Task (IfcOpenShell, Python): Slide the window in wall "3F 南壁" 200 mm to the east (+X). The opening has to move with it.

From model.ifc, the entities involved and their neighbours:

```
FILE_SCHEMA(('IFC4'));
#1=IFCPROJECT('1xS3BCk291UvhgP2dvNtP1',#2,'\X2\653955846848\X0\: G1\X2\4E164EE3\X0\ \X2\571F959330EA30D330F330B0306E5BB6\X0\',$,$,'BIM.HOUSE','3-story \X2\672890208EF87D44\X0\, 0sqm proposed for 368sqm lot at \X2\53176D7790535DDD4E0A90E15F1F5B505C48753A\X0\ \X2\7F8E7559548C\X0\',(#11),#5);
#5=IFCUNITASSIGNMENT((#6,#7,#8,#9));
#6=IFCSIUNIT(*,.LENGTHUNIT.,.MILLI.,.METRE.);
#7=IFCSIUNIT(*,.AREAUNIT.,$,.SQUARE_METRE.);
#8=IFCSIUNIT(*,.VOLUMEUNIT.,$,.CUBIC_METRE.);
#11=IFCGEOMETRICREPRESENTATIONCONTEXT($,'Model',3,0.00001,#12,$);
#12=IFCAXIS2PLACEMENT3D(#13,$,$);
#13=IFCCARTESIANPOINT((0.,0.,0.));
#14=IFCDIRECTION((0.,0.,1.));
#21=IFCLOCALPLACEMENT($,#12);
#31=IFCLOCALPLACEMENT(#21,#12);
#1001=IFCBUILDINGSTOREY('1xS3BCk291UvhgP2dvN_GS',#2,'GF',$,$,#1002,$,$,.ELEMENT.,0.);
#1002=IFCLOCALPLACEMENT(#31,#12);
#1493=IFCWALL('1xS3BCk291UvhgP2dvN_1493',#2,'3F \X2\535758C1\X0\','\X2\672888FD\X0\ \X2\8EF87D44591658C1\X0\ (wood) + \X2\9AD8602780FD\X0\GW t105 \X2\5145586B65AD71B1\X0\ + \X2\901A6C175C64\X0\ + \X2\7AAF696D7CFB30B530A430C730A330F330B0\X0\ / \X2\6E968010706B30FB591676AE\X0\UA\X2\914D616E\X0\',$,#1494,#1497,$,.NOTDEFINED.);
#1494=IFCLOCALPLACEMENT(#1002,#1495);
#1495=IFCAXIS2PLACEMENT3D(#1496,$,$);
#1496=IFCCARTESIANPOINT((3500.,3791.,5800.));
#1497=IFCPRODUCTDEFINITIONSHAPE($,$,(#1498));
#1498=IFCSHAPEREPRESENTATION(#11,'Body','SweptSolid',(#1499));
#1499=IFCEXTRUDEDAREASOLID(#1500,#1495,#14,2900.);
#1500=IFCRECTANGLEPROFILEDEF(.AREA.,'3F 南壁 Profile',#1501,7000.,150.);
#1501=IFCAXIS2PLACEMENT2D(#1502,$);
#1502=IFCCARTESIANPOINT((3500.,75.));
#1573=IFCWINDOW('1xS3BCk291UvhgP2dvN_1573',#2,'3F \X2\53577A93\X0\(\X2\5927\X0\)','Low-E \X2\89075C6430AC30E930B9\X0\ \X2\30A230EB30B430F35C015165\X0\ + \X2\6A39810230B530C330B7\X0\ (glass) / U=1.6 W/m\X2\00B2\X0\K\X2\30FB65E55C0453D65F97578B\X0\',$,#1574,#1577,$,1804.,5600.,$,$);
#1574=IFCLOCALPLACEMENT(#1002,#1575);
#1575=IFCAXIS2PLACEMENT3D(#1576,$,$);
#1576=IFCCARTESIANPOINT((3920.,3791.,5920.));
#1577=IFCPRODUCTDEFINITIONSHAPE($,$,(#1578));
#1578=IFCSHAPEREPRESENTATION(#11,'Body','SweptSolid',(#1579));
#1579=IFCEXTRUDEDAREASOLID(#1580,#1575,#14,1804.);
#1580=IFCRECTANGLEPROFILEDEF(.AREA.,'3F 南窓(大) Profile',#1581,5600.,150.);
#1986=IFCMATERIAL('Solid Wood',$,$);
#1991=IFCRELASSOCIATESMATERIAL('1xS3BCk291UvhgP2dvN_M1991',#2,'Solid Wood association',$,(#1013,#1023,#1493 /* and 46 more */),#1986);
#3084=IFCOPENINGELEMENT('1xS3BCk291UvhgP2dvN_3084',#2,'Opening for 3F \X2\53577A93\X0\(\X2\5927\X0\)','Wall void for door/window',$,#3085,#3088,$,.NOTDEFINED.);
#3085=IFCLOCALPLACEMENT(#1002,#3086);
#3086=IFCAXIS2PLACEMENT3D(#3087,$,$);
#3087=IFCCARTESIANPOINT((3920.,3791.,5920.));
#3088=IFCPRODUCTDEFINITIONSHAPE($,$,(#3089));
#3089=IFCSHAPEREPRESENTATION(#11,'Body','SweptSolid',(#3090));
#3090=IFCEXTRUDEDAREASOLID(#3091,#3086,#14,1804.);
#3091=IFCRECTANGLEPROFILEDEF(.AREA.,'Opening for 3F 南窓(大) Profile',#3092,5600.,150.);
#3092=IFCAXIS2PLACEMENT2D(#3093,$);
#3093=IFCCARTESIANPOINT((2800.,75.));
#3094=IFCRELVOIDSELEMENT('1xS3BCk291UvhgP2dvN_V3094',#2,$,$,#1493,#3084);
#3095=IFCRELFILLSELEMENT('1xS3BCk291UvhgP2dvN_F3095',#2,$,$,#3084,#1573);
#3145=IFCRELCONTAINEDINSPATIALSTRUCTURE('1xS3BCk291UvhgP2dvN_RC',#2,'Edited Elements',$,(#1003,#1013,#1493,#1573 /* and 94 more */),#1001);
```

```python
import ifcopenshell
import ifcopenshell.api.geometry
import ifcopenshell.util.placement
import ifcopenshell.util.unit

model = ifcopenshell.open("model.ifc")
unit_scale = ifcopenshell.util.unit.calculate_unit_scale(model)

window = model.by_guid("1xS3BCk291UvhgP2dvN_1573")
opening = window.FillsVoids[0].RelatingOpeningElement
wall = opening.VoidsElements[0].RelatingBuildingElement

wall_matrix = ifcopenshell.util.placement.get_local_placement(wall.ObjectPlacement)
shift = wall_matrix[:3, 0] * 0.2 / unit_scale
before = ifcopenshell.util.placement.get_local_placement(window.ObjectPlacement)[:3, 3].copy()

# The window is not placed relative to its opening, so move both.
for product in (opening, window):
    matrix = ifcopenshell.util.placement.get_local_placement(product.ObjectPlacement)
    matrix[:3, 3] += shift
    ifcopenshell.api.geometry.edit_object_placement(model, product=product, matrix=matrix, is_si=False)

after = ifcopenshell.util.placement.get_local_placement(window.ObjectPlacement)[:3, 3]
print("window moved by", (after - before).round(3) + 0.0)

model.write("model_updated.ifc")
```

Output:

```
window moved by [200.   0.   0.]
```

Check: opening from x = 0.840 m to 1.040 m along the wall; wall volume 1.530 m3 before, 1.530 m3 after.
